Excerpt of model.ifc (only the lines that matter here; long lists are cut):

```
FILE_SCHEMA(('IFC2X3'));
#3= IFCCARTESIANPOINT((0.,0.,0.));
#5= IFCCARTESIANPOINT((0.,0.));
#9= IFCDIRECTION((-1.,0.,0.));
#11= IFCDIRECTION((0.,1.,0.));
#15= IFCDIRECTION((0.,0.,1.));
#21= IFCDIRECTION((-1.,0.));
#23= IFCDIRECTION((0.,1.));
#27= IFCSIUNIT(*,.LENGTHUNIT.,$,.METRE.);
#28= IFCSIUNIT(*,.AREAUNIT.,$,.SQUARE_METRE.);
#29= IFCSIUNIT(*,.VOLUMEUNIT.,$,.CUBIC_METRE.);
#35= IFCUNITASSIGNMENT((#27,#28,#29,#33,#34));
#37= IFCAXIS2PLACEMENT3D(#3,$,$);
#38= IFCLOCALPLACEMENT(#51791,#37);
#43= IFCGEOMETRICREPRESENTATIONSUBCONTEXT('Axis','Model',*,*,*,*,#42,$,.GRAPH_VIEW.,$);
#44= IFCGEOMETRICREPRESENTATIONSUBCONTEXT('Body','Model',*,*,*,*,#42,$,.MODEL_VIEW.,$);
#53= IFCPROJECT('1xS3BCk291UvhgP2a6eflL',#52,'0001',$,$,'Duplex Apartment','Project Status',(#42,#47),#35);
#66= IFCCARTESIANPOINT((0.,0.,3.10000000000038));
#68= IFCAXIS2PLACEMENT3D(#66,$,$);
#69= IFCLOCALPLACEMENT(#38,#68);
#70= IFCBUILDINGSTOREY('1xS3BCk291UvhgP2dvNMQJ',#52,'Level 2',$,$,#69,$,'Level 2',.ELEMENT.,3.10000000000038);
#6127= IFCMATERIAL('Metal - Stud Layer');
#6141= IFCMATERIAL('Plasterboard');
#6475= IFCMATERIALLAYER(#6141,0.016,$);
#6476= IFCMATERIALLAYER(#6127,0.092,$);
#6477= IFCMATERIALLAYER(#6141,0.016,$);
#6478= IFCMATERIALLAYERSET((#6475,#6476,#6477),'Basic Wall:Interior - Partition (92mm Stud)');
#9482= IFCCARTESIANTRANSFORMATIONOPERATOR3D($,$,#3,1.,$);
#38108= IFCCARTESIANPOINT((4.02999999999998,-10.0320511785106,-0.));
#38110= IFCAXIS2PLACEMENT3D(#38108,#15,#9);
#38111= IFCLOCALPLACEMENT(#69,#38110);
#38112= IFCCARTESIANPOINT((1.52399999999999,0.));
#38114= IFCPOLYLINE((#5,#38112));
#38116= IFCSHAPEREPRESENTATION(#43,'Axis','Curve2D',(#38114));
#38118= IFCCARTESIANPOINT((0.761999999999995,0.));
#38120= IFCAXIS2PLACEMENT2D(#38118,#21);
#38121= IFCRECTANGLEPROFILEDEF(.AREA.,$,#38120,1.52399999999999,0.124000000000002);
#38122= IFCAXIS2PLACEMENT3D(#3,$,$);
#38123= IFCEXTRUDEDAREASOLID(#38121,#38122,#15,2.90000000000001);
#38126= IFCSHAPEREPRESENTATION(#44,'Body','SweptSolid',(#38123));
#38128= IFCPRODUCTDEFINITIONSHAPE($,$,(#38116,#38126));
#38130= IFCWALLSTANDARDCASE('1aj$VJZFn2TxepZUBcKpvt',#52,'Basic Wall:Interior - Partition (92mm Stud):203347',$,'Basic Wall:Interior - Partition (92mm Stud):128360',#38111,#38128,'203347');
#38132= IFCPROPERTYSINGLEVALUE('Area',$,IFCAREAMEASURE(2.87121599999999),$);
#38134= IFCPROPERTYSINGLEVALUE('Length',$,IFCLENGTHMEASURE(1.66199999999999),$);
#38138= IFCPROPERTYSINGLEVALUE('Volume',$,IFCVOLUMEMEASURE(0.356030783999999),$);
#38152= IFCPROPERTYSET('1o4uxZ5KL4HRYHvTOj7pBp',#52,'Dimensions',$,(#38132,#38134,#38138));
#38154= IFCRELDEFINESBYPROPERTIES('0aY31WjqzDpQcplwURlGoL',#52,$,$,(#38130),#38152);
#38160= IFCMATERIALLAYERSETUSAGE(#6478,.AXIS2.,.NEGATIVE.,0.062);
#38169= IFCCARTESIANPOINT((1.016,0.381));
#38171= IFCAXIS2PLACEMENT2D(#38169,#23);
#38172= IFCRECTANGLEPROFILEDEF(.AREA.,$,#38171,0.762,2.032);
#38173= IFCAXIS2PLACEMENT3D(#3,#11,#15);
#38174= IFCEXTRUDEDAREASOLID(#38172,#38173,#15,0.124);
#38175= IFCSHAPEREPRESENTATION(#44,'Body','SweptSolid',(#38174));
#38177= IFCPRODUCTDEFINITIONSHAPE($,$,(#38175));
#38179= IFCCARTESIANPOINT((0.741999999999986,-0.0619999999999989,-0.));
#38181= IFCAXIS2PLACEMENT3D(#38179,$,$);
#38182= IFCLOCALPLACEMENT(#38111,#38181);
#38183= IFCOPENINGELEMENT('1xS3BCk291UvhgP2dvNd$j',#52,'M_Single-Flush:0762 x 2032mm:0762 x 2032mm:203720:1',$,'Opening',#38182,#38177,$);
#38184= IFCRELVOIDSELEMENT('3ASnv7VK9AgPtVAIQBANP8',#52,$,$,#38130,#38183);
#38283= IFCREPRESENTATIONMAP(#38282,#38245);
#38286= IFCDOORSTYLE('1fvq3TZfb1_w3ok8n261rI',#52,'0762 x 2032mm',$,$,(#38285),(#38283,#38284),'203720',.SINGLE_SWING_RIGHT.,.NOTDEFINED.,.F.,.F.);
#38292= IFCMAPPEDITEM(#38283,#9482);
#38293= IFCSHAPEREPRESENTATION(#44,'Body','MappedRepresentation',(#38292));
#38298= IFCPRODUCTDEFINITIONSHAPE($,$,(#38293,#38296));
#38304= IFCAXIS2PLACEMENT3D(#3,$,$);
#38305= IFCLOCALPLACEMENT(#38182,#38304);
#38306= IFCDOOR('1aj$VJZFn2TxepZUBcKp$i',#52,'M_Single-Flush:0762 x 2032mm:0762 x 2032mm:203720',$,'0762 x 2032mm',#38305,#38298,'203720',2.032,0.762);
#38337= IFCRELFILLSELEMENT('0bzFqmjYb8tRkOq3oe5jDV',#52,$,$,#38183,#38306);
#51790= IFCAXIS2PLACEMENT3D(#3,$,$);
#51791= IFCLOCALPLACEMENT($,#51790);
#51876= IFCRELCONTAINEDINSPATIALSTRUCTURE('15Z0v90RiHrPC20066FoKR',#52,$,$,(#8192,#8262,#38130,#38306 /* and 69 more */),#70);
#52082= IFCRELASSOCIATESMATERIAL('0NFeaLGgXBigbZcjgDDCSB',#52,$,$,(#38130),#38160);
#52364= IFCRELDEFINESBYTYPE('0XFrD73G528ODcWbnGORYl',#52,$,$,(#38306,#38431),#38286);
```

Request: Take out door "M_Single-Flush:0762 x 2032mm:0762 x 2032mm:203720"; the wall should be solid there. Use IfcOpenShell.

```python
import ifcopenshell
import ifcopenshell.api.feature
import ifcopenshell.api.pset
import ifcopenshell.api.root
import ifcopenshell.geom
import ifcopenshell.util.element
import ifcopenshell.util.shape
import ifcopenshell.util.unit

model = ifcopenshell.open("model.ifc")
area_scale = ifcopenshell.util.unit.calculate_unit_scale(model, "AREAUNIT")
volume_scale = ifcopenshell.util.unit.calculate_unit_scale(model, "VOLUMEUNIT")
settings = ifcopenshell.geom.settings()


def volume(element):
    """Net volume in cubic metres, openings subtracted."""
    shape = ifcopenshell.geom.create_shape(settings, element)
    return ifcopenshell.util.shape.get_volume(shape.geometry)


door = model.by_guid("1aj$VJZFn2TxepZUBcKp$i")
opening = door.FillsVoids[0].RelatingOpeningElement
wall = opening.VoidsElements[0].RelatingBuildingElement
before = volume(wall)

ifcopenshell.api.root.remove_product(model, product=door)
ifcopenshell.api.feature.remove_feature(model, feature=opening)

after = volume(wall)
thickness = 0.124  # wall thickness in metres

# Update the wall's stored quantities.
pset = model.by_id(ifcopenshell.util.element.get_pset(wall, "Dimensions", should_inherit=False)["id"])
ifcopenshell.api.pset.edit_pset(model, pset=pset, properties={
    "Area": model.create_entity("IfcAreaMeasure", after / thickness / area_scale),
    "Volume": model.create_entity("IfcVolumeMeasure", after / volume_scale),
})

print(f"wall volume {before:.3f} -> {after:.3f} m3")

model.write("model-out.ifc")
```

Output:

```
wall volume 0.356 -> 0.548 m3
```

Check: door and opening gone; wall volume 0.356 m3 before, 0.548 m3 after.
